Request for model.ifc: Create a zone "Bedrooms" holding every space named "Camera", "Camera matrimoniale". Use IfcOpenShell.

First a look at what the model holds.

```python
import ifcopenshell

model = ifcopenshell.open("model.ifc")
print(model.schema)
seen = {}
for space in model.by_type("IfcSpace"):
    seen[space.LongName] = seen.get(space.LongName, 0) + 1
for name, count in sorted(seen.items(), key=str):
    print(count, "x", name)
print("zones:", [z.Name for z in model.by_type("IfcZone")][:20])
```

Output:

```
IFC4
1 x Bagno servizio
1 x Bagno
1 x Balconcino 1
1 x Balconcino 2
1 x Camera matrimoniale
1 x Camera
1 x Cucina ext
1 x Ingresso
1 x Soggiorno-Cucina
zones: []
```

```python
import ifcopenshell
import ifcopenshell.api.group
import ifcopenshell.api.root

model = ifcopenshell.open("model.ifc")

names = {"Camera", "Camera matrimoniale"}
spaces = [s for s in model.by_type("IfcSpace") if s.LongName in names]

zone = ifcopenshell.api.root.create_entity(model, ifc_class="IfcZone", name="Bedrooms")
ifcopenshell.api.group.assign_group(model, products=spaces, group=zone)
print(len(spaces), "spaces in", zone.Name)

model.write("model_edited.ifc")
```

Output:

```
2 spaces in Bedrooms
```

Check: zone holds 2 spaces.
